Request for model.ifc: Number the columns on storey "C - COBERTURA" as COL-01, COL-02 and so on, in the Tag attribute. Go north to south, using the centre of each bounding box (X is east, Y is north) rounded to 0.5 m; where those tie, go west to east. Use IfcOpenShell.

First a look at what the model holds.

```python
import ifcopenshell
import ifcopenshell.util.element
import ifcopenshell.util.placement

model = ifcopenshell.open("model.ifc")
print(model.schema)
storey = next(s for s in model.by_type("IfcBuildingStorey") if s.Name == "C - COBERTURA")
columns = [e for e in ifcopenshell.util.element.get_decomposition(storey) if e.is_a("IfcColumn")]
for e in sorted(columns, key=lambda e: e.id()):
    origin = ifcopenshell.util.placement.get_local_placement(e.ObjectPlacement)[:3, 3]
    print(e.id(), e.Tag, e.Name, origin.round(2) + 0.0, sep=" | ")
```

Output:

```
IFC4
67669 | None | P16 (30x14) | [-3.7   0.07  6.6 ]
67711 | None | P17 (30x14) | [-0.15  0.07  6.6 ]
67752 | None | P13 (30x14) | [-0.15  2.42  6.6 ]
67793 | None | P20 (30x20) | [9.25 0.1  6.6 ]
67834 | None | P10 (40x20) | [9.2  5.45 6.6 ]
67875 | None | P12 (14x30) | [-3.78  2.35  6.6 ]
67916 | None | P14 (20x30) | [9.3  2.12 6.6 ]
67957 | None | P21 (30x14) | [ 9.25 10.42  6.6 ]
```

```python
import ifcopenshell
import ifcopenshell.geom
import ifcopenshell.util.element
import ifcopenshell.util.shape

model = ifcopenshell.open("model.ifc")
settings = ifcopenshell.geom.settings()
settings.set("use-world-coords", True)


def centre(element):
    shape = ifcopenshell.geom.create_shape(settings, element)
    return ifcopenshell.util.shape.get_bbox_centroid(shape.geometry)


storey = next(s for s in model.by_type("IfcBuildingStorey") if s.Name == "C - COBERTURA")
columns = [e for e in ifcopenshell.util.element.get_decomposition(storey) if e.is_a("IfcColumn")]

# Insertion points can sit at a corner or the storey origin, so sort by the geometry (in metres).
centres = {e: centre(e) for e in columns}
columns.sort(key=lambda e: (-round(centres[e][1] / 0.5), centres[e][0]))

for i, e in enumerate(columns, start=1):
    number = f"COL-{i:02d}"
    e.Tag = number
    print(e.id(), number)

model.write("model_rev.ifc")
```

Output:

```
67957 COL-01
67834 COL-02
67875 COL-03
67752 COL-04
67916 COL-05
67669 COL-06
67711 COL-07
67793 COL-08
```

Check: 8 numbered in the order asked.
